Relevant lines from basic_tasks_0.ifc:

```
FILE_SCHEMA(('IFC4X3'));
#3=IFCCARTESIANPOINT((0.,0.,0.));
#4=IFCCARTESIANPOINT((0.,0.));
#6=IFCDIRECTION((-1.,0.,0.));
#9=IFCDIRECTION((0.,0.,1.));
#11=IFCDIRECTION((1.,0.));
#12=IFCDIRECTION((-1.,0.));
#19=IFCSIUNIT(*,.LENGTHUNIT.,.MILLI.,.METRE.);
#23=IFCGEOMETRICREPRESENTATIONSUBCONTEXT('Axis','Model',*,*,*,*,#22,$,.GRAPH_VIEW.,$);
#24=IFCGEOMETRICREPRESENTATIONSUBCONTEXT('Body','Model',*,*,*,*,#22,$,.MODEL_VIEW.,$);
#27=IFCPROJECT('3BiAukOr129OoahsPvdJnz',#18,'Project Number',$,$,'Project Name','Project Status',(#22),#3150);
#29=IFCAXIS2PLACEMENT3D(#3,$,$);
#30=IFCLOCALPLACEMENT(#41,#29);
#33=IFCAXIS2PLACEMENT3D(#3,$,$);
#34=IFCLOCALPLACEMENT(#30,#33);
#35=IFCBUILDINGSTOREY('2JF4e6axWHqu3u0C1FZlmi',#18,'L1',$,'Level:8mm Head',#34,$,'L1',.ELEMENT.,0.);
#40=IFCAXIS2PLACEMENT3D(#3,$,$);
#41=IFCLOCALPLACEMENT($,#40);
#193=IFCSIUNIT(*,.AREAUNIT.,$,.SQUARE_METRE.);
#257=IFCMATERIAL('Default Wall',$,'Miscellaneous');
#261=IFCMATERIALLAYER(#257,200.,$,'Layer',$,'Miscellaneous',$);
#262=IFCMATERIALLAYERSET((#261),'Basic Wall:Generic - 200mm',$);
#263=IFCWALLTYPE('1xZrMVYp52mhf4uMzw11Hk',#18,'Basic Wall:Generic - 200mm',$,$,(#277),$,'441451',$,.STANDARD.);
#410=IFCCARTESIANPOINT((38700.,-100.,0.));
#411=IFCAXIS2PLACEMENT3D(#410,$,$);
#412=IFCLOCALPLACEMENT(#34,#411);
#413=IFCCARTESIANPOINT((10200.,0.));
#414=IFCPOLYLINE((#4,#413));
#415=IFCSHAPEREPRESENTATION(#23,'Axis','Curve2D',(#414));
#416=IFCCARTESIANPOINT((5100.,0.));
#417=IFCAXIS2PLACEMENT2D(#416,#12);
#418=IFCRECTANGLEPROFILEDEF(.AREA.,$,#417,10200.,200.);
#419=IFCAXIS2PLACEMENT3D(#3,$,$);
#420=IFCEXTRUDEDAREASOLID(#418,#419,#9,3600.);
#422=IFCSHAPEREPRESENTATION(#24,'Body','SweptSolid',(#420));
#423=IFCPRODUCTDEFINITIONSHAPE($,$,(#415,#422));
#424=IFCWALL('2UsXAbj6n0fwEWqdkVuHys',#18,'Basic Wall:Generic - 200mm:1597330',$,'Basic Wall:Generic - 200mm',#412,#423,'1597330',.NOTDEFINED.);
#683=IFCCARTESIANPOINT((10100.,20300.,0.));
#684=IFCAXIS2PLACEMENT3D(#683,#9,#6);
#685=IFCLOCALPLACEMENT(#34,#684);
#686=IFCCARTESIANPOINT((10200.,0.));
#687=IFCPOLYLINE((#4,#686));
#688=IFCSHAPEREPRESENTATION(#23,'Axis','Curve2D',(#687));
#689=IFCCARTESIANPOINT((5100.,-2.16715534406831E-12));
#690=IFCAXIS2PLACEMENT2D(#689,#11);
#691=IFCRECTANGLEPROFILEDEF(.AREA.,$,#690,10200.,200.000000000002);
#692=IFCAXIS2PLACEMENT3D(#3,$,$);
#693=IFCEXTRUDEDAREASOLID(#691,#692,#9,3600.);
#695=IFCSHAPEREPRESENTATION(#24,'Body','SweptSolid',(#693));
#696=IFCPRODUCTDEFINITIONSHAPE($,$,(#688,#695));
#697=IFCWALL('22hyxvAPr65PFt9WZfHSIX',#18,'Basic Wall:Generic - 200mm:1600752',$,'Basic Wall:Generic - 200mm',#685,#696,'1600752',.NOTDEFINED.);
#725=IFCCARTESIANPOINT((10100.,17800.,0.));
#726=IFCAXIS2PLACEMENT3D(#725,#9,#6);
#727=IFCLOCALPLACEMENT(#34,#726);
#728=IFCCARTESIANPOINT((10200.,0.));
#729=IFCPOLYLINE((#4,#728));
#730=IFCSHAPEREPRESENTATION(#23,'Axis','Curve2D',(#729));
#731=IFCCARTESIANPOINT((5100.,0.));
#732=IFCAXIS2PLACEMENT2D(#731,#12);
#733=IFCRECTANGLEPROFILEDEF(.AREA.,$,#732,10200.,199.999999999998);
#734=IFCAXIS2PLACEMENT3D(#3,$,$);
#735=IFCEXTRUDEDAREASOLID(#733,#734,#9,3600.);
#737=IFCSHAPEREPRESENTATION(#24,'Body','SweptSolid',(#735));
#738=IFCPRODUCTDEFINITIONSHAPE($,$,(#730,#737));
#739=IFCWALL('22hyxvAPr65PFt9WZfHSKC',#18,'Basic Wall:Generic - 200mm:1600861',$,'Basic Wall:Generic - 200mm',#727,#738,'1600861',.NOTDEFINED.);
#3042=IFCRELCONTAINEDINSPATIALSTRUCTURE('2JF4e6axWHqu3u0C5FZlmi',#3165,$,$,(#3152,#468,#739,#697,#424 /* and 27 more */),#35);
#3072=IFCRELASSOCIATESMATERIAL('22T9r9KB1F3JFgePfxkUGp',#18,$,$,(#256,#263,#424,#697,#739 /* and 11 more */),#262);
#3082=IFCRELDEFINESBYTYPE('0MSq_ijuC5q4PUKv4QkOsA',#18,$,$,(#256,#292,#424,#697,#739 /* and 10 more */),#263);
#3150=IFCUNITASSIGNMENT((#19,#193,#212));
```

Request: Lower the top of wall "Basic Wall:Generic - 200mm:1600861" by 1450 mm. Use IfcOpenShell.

```python
import ifcopenshell
import ifcopenshell.geom
import ifcopenshell.util.representation
import ifcopenshell.util.shape
import ifcopenshell.util.unit

model = ifcopenshell.open("basic_tasks_0.ifc")
unit_scale = ifcopenshell.util.unit.calculate_unit_scale(model)
settings = ifcopenshell.geom.settings()


def volume(element):
    """Net volume in cubic metres, openings subtracted."""
    shape = ifcopenshell.geom.create_shape(settings, element)
    return ifcopenshell.util.shape.get_volume(shape.geometry)


wall = model.by_id(739)
before = volume(wall)

body = ifcopenshell.util.representation.get_representation(wall, "Model", "Body")
solid = body.Items[0]
old_height = solid.Depth
solid.Depth -= 1.45 / unit_scale
after = volume(wall)

print(f"height {old_height:g} -> {solid.Depth:g}, volume {before:.3f} -> {after:.3f} m3")

model.write("basic_tasks_0_rev.ifc")
```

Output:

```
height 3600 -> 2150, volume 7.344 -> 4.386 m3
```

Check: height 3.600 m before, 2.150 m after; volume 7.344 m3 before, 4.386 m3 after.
